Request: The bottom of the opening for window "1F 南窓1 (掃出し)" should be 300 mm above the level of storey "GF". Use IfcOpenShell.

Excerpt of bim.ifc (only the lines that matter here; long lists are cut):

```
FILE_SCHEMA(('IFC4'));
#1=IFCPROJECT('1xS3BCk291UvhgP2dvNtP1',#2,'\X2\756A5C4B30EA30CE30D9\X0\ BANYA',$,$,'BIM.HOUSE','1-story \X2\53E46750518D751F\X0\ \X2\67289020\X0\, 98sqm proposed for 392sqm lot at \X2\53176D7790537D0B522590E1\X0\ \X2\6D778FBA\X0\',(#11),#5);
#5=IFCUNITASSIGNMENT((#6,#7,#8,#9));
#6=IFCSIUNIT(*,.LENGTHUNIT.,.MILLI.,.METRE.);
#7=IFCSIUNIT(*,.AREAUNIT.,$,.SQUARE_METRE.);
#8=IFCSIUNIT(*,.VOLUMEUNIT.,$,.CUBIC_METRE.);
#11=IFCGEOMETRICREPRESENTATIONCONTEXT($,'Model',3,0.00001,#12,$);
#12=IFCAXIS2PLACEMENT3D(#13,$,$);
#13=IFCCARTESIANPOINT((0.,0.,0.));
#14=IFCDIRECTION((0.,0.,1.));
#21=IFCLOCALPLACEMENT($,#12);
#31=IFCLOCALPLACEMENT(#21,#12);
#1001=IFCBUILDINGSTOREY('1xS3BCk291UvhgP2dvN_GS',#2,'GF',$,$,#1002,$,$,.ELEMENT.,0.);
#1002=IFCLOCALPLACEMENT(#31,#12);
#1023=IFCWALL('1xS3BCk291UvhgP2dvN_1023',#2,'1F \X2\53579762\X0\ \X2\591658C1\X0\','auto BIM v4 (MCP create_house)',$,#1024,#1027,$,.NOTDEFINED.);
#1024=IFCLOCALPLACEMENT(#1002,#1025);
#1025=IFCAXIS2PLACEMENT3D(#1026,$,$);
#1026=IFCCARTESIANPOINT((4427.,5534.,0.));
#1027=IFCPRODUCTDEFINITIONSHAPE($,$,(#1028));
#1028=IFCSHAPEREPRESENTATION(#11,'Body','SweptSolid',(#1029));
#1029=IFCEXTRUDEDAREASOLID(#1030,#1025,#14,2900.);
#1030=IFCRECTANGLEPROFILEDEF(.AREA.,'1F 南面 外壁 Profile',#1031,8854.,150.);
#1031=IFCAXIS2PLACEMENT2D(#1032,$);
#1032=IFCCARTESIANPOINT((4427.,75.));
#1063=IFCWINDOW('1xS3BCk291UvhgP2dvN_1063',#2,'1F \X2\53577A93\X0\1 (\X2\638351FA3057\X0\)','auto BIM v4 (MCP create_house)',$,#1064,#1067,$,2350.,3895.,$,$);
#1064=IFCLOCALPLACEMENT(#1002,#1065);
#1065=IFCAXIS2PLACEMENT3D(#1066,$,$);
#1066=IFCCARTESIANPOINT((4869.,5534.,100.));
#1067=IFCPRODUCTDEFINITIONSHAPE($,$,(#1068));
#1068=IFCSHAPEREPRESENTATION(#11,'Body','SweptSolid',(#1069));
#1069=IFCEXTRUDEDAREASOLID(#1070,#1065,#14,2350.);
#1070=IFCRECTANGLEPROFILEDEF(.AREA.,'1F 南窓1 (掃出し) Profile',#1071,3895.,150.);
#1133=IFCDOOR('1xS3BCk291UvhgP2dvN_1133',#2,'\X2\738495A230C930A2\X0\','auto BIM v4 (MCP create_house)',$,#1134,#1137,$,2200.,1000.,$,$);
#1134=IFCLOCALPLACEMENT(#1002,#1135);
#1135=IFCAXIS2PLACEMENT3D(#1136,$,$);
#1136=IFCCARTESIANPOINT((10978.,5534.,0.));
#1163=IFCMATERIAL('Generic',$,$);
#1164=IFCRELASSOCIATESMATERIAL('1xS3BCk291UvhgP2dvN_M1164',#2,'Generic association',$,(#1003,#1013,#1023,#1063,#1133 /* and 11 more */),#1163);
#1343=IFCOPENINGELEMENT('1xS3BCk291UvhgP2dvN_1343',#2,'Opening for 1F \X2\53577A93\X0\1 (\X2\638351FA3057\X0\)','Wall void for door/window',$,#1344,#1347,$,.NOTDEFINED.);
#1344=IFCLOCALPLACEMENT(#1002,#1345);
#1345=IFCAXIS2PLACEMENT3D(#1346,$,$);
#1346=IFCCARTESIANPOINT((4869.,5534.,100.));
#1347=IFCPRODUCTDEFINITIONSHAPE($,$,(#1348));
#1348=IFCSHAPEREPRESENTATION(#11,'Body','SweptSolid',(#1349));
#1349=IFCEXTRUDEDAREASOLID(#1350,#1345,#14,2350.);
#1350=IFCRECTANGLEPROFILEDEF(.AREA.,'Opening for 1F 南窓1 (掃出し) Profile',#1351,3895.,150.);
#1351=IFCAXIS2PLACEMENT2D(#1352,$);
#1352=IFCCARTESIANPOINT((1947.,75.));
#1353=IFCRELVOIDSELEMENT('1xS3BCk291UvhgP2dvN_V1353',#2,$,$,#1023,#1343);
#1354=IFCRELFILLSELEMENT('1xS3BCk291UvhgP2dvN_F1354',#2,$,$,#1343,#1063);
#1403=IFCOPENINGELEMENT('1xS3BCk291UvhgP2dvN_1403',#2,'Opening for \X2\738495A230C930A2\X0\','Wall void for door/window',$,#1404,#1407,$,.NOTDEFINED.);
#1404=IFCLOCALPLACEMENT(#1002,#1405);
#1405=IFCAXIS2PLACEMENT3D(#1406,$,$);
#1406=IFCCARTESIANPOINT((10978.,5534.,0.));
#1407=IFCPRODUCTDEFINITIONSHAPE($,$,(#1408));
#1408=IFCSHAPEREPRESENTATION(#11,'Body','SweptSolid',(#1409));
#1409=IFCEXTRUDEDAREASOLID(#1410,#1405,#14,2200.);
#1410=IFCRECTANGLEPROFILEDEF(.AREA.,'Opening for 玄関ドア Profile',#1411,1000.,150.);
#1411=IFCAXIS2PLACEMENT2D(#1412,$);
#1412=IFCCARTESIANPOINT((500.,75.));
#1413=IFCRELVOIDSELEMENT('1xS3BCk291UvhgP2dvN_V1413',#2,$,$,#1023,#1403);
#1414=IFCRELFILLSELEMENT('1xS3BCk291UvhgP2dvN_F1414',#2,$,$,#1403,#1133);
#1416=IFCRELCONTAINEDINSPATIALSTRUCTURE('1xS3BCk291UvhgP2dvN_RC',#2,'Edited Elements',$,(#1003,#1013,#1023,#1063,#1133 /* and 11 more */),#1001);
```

```python
import numpy as np
import ifcopenshell
import ifcopenshell.api.geometry
import ifcopenshell.geom
import ifcopenshell.util.element
import ifcopenshell.util.placement
import ifcopenshell.util.shape
import ifcopenshell.util.unit

model = ifcopenshell.open("bim.ifc")
unit_scale = ifcopenshell.util.unit.calculate_unit_scale(model)

window = model.by_guid("1xS3BCk291UvhgP2dvN_1063")
opening = window.FillsVoids[0].RelatingOpeningElement
storey = ifcopenshell.util.element.get_container(window, ifc_class="IfcBuildingStorey")
level = ifcopenshell.util.placement.get_local_placement(storey.ObjectPlacement)[2, 3]

# The opening's origin need not be at the sill, so measure its lowest point.
shape = ifcopenshell.geom.create_shape(ifcopenshell.geom.settings(), opening)
bottom = ifcopenshell.util.shape.get_shape_bottom_elevation(shape, shape.geometry) / unit_scale
dz = level + 0.3 / unit_scale - bottom

shift = np.array([0.0, 0.0, dz])
# The window is not placed relative to its opening, so move both.
for product in (opening, window):
    matrix = ifcopenshell.util.placement.get_local_placement(product.ObjectPlacement)
    matrix[:3, 3] += shift
    ifcopenshell.api.geometry.edit_object_placement(model, product=product, matrix=matrix, is_si=False)

print(f"moved by {dz * unit_scale:+.3f} m")

model.write("bim_v2.ifc")
```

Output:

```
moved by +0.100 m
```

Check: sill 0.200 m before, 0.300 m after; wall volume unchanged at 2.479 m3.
